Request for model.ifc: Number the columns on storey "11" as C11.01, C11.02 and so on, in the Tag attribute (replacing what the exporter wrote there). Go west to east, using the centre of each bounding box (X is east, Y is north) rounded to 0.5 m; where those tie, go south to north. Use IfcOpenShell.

First a look at what the model holds.

```python
import ifcopenshell
import ifcopenshell.util.element
import ifcopenshell.util.placement

model = ifcopenshell.open("model.ifc")
print(model.schema)
storey = next(s for s in model.by_type("IfcBuildingStorey") if s.Name == "11")
columns = [e for e in ifcopenshell.util.element.get_decomposition(storey) if e.is_a("IfcColumn")]
for e in sorted(columns, key=lambda e: e.id()):
    origin = ifcopenshell.util.placement.get_local_placement(e.ObjectPlacement)[:3, 3]
    print(e.id(), e.Tag, e.Name, origin.round(2) + 0.0, sep=" | ")
```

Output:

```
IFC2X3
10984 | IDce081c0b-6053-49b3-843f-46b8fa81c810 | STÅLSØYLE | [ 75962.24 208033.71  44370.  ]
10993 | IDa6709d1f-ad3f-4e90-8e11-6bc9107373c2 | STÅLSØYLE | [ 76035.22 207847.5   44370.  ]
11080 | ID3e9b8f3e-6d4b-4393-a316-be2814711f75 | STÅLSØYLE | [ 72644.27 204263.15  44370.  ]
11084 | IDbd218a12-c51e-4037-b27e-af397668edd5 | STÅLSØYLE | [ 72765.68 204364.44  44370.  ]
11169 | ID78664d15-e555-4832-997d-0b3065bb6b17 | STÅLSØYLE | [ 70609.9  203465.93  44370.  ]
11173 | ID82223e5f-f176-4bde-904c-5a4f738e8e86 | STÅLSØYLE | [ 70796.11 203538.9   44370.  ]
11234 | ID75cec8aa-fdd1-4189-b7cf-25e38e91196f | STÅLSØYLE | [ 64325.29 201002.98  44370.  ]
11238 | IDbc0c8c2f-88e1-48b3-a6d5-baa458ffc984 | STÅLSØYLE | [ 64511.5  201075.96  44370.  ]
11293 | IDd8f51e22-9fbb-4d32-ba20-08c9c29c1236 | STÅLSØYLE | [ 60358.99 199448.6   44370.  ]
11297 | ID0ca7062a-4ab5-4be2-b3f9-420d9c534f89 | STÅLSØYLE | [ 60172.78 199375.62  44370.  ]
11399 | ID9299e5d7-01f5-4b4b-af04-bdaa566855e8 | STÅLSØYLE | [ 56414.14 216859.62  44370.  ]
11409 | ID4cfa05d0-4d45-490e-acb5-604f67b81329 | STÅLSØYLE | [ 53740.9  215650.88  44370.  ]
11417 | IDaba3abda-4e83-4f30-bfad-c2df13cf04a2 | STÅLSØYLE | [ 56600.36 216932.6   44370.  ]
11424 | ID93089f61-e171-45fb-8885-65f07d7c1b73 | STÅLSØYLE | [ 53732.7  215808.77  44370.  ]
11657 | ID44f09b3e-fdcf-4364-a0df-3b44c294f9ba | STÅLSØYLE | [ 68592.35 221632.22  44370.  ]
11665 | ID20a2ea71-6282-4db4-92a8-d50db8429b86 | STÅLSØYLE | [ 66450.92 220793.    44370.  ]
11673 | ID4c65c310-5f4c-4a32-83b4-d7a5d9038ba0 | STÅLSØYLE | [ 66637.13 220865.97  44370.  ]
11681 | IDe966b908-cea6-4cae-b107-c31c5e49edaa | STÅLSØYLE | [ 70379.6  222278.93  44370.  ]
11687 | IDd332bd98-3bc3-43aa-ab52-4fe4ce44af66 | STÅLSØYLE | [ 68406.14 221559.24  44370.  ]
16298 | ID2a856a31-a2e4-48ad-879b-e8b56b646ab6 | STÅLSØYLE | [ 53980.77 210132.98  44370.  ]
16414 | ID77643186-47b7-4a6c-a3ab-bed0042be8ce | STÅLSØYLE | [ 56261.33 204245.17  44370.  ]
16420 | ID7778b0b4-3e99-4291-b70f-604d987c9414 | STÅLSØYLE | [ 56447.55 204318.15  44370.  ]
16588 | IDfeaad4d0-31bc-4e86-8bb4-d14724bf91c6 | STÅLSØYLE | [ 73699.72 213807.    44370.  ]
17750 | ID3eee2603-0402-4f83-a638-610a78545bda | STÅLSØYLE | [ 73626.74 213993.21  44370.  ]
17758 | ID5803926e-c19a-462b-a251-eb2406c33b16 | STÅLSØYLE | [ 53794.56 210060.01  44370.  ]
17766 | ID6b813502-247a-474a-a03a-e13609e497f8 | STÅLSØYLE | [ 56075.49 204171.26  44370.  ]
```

```python
import ifcopenshell
import ifcopenshell.geom
import ifcopenshell.util.element
import ifcopenshell.util.shape

model = ifcopenshell.open("model.ifc")
settings = ifcopenshell.geom.settings()
settings.set("use-world-coords", True)


def centre(element):
    shape = ifcopenshell.geom.create_shape(settings, element)
    return ifcopenshell.util.shape.get_bbox_centroid(shape.geometry)


storey = next(s for s in model.by_type("IfcBuildingStorey") if s.Name == "11")
columns = [e for e in ifcopenshell.util.element.get_decomposition(storey) if e.is_a("IfcColumn")]

# Insertion points can sit at a corner or the storey origin, so sort by the geometry (in metres).
centres = {e: centre(e) for e in columns}
columns.sort(key=lambda e: (round(centres[e][0] / 0.5), centres[e][1]))

for i, e in enumerate(columns, start=1):
    number = f"C11.{i:02d}"
    e.Tag = number
    print(e.id(), number)

model.write("model_rev.ifc")
```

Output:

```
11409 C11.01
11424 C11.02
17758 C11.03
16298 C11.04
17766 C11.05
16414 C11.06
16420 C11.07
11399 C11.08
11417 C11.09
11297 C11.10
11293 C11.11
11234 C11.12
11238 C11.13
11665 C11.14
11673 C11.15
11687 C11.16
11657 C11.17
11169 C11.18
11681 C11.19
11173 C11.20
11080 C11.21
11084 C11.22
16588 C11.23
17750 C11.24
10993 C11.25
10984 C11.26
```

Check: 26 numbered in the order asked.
